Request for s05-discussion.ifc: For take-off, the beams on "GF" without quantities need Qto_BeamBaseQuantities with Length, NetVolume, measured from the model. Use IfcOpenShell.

First a look at what the model holds.

```python
import ifcopenshell
import ifcopenshell.util.element
import ifcopenshell.util.unit

model = ifcopenshell.open("s05-discussion.ifc")
print(model.schema)
for unit_type in ("LENGTHUNIT", "AREAUNIT", "VOLUMEUNIT"):
    print(unit_type, ifcopenshell.util.unit.calculate_unit_scale(model, unit_type))
storey = next(s for s in model.by_type("IfcBuildingStorey") if s.Name == "GF")
beams = [e for e in ifcopenshell.util.element.get_decomposition(storey) if e.is_a("IfcBeam")]
for e in sorted(beams, key=lambda e: e.id()):
    print(e.id(), e.is_a(), e.Name, list(ifcopenshell.util.element.get_psets(e, qtos_only=True)), sep=" | ")
```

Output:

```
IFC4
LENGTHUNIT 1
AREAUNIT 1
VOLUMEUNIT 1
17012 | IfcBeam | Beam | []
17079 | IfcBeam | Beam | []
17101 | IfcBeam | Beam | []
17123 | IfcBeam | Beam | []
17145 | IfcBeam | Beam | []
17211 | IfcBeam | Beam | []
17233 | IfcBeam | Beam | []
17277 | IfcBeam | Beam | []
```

```python
import ifcopenshell
import ifcopenshell.api.pset
import ifcopenshell.geom
import ifcopenshell.util.element
import ifcopenshell.util.shape
import ifcopenshell.util.unit

model = ifcopenshell.open("s05-discussion.ifc")
unit_scale = ifcopenshell.util.unit.calculate_unit_scale(model)
volume_scale = ifcopenshell.util.unit.calculate_unit_scale(model, "VOLUMEUNIT")
settings = ifcopenshell.geom.settings()

storey = next(s for s in model.by_type("IfcBuildingStorey") if s.Name == "GF")
beams = [e for e in ifcopenshell.util.element.get_decomposition(storey) if e.is_a("IfcBeam")]

for e in sorted(beams, key=lambda e: e.id()):
    if ifcopenshell.util.element.get_psets(e, qtos_only=True, should_inherit=False):
        continue
    # Geometry comes back in metres, in the element's own axes.
    shape = ifcopenshell.geom.create_shape(settings, e)
    values = {
        "Length": ifcopenshell.util.shape.get_max_xyz(shape.geometry) / unit_scale,
        "NetVolume": ifcopenshell.util.shape.get_volume(shape.geometry) / volume_scale,
    }
    qto = ifcopenshell.api.pset.add_qto(model, product=e, name="Qto_BeamBaseQuantities")
    ifcopenshell.api.pset.edit_qto(model, qto=qto, properties=values)
    print(e.id(), {k: round(v, 3) for k, v in values.items()})

model.write("s05-discussion_v2.ifc")
```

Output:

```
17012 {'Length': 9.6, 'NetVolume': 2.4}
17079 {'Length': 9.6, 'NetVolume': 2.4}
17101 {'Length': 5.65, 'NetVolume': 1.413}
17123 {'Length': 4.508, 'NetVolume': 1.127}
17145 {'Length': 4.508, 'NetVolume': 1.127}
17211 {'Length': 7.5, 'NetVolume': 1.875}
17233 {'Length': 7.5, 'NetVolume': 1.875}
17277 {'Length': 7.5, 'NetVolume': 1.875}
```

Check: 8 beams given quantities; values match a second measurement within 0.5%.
